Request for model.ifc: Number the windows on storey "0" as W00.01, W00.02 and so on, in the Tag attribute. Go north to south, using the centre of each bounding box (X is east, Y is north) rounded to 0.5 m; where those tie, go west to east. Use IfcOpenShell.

First a look at what the model holds.

```python
import ifcopenshell
import ifcopenshell.util.element
import ifcopenshell.util.placement

model = ifcopenshell.open("model.ifc")
print(model.schema)
storey = next(s for s in model.by_type("IfcBuildingStorey") if s.Name == "0")
windows = [e for e in ifcopenshell.util.element.get_decomposition(storey) if e.is_a("IfcWindow")]
for e in sorted(windows, key=lambda e: e.id()):
    origin = ifcopenshell.util.placement.get_local_placement(e.ObjectPlacement)[:3, 3]
    print(e.id(), e.Tag, e.Name, origin.round(2) + 0.0, sep=" | ")
```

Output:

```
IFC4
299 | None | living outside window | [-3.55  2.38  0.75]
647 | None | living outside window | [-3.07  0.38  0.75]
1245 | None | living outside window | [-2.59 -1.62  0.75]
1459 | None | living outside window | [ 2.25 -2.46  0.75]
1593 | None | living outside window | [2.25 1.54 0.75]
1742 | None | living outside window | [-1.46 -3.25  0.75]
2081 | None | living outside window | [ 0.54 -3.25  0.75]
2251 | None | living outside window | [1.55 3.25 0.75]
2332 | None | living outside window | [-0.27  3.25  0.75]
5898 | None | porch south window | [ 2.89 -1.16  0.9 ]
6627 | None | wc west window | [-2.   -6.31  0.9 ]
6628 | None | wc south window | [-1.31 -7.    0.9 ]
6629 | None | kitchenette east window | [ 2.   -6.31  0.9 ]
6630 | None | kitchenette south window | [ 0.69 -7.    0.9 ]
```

```python
import ifcopenshell
import ifcopenshell.geom
import ifcopenshell.util.element
import ifcopenshell.util.shape

model = ifcopenshell.open("model.ifc")
settings = ifcopenshell.geom.settings()
settings.set("use-world-coords", True)


def centre(element):
    shape = ifcopenshell.geom.create_shape(settings, element)
    return ifcopenshell.util.shape.get_bbox_centroid(shape.geometry)


storey = next(s for s in model.by_type("IfcBuildingStorey") if s.Name == "0")
windows = [e for e in ifcopenshell.util.element.get_decomposition(storey) if e.is_a("IfcWindow")]

# Insertion points can sit at a corner or the storey origin, so sort by the geometry (in metres).
centres = {e: centre(e) for e in windows}
windows.sort(key=lambda e: (-round(centres[e][1] / 0.5), centres[e][0]))

for i, e in enumerate(windows, start=1):
    number = f"W00.{i:02d}"
    e.Tag = number
    print(e.id(), number)

model.write("model_rev.ifc")
```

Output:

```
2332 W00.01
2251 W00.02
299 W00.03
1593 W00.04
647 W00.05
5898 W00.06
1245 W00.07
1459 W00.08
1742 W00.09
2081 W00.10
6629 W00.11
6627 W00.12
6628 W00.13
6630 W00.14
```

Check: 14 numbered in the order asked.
